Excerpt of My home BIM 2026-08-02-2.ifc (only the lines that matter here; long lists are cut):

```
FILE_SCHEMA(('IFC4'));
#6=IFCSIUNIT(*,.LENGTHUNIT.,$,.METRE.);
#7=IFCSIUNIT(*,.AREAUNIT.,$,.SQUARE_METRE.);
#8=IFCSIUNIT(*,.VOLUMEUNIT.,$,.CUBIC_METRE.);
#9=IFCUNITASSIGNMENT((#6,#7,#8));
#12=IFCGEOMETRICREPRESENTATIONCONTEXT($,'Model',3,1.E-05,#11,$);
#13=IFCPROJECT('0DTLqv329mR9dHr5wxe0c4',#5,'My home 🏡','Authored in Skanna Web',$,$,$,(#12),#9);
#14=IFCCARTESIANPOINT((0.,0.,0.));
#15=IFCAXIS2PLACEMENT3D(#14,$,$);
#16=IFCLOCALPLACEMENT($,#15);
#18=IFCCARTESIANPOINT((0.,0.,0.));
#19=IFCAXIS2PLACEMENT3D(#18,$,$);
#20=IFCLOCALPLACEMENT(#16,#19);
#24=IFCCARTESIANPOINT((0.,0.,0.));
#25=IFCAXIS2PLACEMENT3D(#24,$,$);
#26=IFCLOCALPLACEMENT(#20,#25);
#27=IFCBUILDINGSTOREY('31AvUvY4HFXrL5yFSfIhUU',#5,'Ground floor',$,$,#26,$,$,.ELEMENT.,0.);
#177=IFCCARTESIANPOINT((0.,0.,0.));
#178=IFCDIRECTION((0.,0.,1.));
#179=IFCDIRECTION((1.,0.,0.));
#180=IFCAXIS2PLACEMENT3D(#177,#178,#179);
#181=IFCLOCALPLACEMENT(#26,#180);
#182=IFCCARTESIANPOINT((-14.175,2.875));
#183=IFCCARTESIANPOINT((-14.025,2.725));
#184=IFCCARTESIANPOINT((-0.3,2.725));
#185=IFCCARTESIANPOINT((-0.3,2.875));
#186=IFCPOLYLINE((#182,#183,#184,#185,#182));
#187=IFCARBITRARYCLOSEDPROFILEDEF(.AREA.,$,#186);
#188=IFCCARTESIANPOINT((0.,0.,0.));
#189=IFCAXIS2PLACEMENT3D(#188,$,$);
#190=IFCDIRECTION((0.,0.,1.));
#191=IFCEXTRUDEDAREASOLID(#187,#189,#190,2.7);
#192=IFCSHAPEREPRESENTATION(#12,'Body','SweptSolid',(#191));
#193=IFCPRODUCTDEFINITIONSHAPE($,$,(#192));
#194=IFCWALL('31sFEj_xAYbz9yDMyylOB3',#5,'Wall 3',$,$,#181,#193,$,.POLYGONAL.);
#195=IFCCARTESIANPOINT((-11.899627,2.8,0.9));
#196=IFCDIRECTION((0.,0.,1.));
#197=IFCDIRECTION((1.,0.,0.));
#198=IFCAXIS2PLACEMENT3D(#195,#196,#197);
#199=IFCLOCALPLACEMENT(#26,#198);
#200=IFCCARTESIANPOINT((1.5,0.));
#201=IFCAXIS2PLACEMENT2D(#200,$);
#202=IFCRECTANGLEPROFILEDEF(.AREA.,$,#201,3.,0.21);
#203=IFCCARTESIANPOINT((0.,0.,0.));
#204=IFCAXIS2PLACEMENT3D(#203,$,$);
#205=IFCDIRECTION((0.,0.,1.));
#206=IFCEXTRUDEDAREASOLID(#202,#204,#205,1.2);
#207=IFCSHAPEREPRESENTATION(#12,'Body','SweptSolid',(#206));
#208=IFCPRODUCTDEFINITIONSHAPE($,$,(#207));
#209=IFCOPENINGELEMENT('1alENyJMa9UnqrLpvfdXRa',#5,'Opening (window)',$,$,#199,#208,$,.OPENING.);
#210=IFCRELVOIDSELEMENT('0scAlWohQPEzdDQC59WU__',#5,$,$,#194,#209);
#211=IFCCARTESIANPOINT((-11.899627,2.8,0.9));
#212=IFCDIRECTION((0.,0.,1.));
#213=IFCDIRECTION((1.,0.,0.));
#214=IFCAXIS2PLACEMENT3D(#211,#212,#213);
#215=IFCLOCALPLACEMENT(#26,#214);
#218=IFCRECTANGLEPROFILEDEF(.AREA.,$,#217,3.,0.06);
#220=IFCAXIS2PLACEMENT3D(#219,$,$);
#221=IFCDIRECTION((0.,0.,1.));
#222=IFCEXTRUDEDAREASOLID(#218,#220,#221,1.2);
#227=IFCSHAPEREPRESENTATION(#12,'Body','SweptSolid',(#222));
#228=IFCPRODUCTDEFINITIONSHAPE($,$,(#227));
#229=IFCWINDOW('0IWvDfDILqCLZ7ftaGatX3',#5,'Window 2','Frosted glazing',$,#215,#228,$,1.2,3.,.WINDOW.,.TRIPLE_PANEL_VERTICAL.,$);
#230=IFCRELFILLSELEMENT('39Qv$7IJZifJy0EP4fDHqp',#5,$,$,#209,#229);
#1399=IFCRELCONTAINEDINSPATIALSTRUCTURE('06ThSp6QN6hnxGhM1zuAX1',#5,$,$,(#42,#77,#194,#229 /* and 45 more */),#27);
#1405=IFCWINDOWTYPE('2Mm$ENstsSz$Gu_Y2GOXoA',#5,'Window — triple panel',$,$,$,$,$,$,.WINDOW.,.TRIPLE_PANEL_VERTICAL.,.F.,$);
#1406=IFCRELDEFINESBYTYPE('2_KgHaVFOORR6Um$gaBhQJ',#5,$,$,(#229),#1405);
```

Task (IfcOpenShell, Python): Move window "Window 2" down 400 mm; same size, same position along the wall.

```python
import numpy as np
import ifcopenshell
import ifcopenshell.api.geometry
import ifcopenshell.util.placement
import ifcopenshell.util.unit

model = ifcopenshell.open("My home BIM 2026-08-02-2.ifc")
unit_scale = ifcopenshell.util.unit.calculate_unit_scale(model)

window = model.by_guid("0IWvDfDILqCLZ7ftaGatX3")
opening = window.FillsVoids[0].RelatingOpeningElement
dz = -0.4

shift = np.array([0.0, 0.0, dz])
# The window is not placed relative to its opening, so move both.
for product in (opening, window):
    matrix = ifcopenshell.util.placement.get_local_placement(product.ObjectPlacement)
    matrix[:3, 3] += shift
    ifcopenshell.api.geometry.edit_object_placement(model, product=product, matrix=matrix, is_si=False)

print(f"moved by {dz * unit_scale:+.3f} m")

model.write("My home BIM 2026-08-02-2-out.ifc")
```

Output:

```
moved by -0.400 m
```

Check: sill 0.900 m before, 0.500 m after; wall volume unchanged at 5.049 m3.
